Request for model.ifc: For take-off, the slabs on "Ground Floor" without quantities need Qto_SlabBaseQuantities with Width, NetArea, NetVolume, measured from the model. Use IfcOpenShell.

First a look at what the model holds.

```python
import ifcopenshell
import ifcopenshell.util.element
import ifcopenshell.util.unit

model = ifcopenshell.open("model.ifc")
print(model.schema)
for unit_type in ("LENGTHUNIT", "AREAUNIT", "VOLUMEUNIT"):
    print(unit_type, ifcopenshell.util.unit.calculate_unit_scale(model, unit_type))
storey = next(s for s in model.by_type("IfcBuildingStorey") if s.Name == "Ground Floor")
slabs = [e for e in ifcopenshell.util.element.get_decomposition(storey) if e.is_a("IfcSlab")]
for e in sorted(slabs, key=lambda e: e.id()):
    print(e.id(), e.is_a(), e.Name, list(ifcopenshell.util.element.get_psets(e, qtos_only=True)), sep=" | ")
```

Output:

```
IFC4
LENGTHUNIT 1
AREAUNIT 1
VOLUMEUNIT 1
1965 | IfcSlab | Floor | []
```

```python
import ifcopenshell
import ifcopenshell.api.pset
import ifcopenshell.geom
import ifcopenshell.util.element
import ifcopenshell.util.shape
import ifcopenshell.util.unit

model = ifcopenshell.open("model.ifc")
unit_scale = ifcopenshell.util.unit.calculate_unit_scale(model)
area_scale = ifcopenshell.util.unit.calculate_unit_scale(model, "AREAUNIT")
volume_scale = ifcopenshell.util.unit.calculate_unit_scale(model, "VOLUMEUNIT")
settings = ifcopenshell.geom.settings()

storey = next(s for s in model.by_type("IfcBuildingStorey") if s.Name == "Ground Floor")
slabs = [e for e in ifcopenshell.util.element.get_decomposition(storey) if e.is_a("IfcSlab")]

for e in sorted(slabs, key=lambda e: e.id()):
    if ifcopenshell.util.element.get_psets(e, qtos_only=True, should_inherit=False):
        continue
    # Geometry comes back in metres, in the element's own axes.
    shape = ifcopenshell.geom.create_shape(settings, e)
    values = {
        "Width": ifcopenshell.util.shape.get_z(shape.geometry) / unit_scale,
        "NetArea": ifcopenshell.util.shape.get_footprint_area(shape.geometry) / area_scale,
        "NetVolume": ifcopenshell.util.shape.get_volume(shape.geometry) / volume_scale,
    }
    qto = ifcopenshell.api.pset.add_qto(model, product=e, name="Qto_SlabBaseQuantities")
    ifcopenshell.api.pset.edit_qto(model, qto=qto, properties=values)
    print(e.id(), {k: round(v, 3) for k, v in values.items()})

model.write("model_edited.ifc")
```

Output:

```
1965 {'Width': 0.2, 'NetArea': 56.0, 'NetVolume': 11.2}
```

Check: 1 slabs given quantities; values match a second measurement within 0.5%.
